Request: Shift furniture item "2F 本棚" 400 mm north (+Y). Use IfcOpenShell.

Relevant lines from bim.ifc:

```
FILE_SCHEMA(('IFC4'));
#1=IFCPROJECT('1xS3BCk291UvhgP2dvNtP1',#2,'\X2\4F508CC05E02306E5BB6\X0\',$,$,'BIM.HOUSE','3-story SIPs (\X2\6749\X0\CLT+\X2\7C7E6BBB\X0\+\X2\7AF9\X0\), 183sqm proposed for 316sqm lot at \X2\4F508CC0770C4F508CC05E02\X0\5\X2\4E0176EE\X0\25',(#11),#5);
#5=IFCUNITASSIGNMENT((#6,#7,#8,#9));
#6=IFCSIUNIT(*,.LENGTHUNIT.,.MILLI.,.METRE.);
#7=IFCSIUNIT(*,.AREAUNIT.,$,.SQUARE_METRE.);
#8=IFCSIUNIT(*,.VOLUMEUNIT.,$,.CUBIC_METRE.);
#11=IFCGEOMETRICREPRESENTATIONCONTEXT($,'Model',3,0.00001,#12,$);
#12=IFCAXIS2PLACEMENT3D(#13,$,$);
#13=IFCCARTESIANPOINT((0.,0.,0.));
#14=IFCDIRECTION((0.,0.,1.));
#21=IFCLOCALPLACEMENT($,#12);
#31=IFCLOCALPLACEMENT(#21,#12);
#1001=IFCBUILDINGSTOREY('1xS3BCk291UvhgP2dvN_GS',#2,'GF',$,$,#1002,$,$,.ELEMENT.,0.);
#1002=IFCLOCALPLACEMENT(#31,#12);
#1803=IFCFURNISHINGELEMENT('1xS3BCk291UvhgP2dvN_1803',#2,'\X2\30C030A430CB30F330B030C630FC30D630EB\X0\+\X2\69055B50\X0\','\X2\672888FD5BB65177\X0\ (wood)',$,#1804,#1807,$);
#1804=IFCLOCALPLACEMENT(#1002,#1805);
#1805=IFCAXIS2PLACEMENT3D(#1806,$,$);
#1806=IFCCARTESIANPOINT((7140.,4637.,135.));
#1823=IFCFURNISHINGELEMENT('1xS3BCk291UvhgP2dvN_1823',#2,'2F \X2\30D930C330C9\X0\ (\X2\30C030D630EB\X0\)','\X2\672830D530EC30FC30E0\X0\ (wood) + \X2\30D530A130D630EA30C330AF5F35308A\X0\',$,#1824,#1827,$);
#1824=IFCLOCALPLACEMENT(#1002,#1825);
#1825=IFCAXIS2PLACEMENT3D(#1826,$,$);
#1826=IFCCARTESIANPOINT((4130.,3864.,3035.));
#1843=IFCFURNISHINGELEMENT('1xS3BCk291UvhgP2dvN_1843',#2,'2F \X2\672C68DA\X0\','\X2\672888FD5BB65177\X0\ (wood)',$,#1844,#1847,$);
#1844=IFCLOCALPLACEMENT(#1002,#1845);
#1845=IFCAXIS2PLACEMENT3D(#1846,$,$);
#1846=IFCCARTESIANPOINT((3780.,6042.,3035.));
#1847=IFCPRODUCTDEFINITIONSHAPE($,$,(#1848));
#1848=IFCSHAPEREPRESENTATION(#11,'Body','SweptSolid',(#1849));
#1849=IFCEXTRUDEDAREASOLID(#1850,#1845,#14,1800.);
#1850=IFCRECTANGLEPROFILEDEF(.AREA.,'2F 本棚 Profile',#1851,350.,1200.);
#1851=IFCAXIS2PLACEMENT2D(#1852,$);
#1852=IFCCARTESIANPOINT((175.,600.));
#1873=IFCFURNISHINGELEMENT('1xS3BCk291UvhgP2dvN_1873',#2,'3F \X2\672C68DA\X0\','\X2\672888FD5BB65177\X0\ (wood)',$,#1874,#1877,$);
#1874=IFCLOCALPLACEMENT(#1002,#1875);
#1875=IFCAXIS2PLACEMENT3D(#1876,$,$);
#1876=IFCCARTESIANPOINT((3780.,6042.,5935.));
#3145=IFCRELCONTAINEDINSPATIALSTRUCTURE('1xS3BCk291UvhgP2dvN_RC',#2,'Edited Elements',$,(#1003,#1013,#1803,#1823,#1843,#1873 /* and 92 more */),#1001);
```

```python
import ifcopenshell
import ifcopenshell.api.geometry
import ifcopenshell.util.placement
import ifcopenshell.util.unit

model = ifcopenshell.open("bim.ifc")
unit_scale = ifcopenshell.util.unit.calculate_unit_scale(model)

item = model.by_guid("1xS3BCk291UvhgP2dvN_1843")
matrix = ifcopenshell.util.placement.get_local_placement(item.ObjectPlacement)
matrix[1, 3] += 0.4 / unit_scale
ifcopenshell.api.geometry.edit_object_placement(model, product=item, matrix=matrix, is_si=False)

print(ifcopenshell.util.placement.get_local_placement(item.ObjectPlacement).round(3) + 0.0)

model.write("bim_updated.ifc")
```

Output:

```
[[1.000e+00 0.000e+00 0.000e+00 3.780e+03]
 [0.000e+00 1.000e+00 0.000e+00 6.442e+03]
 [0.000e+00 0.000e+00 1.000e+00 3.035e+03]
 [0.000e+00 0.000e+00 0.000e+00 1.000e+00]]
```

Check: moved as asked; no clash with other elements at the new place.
